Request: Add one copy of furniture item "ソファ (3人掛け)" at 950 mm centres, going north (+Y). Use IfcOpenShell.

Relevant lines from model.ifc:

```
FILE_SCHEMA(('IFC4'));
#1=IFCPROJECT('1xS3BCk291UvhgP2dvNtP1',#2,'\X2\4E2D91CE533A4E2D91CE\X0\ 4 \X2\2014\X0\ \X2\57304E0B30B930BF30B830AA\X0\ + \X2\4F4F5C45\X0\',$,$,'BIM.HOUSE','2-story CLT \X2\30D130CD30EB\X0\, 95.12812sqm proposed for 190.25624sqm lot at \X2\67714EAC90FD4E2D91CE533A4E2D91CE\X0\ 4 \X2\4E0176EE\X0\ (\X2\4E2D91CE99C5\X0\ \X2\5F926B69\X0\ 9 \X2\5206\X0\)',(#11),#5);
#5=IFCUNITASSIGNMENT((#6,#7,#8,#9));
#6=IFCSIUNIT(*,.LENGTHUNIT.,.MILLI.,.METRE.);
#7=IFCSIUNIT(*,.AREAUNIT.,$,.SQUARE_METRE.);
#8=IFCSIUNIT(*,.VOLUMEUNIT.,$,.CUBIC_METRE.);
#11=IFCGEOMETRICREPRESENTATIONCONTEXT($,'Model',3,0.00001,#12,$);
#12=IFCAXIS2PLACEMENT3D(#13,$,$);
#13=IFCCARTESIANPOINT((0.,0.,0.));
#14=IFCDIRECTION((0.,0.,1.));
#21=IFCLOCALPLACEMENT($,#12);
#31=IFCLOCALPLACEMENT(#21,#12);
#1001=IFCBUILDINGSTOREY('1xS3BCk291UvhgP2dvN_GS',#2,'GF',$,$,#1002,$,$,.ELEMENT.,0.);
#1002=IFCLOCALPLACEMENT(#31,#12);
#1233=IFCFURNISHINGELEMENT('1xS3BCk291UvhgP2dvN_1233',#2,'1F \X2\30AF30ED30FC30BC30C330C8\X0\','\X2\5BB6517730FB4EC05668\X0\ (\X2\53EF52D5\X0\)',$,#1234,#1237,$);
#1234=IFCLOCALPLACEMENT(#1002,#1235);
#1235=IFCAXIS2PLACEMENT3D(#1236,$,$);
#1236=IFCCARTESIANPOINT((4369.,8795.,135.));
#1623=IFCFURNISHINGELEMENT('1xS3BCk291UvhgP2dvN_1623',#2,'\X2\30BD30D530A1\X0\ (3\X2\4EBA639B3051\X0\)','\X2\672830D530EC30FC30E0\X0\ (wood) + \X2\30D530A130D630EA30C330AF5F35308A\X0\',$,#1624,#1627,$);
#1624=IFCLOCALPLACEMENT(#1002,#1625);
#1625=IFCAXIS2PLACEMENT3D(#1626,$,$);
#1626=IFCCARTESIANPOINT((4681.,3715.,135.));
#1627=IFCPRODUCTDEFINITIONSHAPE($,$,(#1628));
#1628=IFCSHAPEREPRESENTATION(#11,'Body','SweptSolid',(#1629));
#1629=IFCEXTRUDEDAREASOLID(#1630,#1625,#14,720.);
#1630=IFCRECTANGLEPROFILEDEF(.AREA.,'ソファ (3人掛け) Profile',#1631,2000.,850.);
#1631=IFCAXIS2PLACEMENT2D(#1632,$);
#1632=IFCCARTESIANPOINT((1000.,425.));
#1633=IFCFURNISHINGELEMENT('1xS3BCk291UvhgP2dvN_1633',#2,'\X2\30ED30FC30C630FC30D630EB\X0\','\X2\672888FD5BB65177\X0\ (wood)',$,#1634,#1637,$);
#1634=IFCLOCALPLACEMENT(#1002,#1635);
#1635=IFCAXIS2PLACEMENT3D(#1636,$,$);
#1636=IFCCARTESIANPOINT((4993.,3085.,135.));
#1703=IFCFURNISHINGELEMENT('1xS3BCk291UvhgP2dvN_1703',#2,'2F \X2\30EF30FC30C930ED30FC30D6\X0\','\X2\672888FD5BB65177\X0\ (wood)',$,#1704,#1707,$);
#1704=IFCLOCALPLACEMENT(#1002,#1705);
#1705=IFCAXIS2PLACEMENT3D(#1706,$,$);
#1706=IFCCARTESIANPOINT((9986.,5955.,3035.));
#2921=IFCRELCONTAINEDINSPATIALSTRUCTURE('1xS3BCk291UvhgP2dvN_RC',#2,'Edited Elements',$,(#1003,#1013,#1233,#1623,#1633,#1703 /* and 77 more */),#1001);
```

```python
import numpy as np
import ifcopenshell
import ifcopenshell.api.geometry
import ifcopenshell.api.root
import ifcopenshell.util.element
import ifcopenshell.util.placement

model = ifcopenshell.open("model.ifc")


def reuse_history(source, copy):
    """copy_class also copies each property set's owner history, people and application; keep the originals."""
    for rel in copy.IsDefinedBy:
        if rel.is_a("IfcRelDefinesByProperties") and (history := rel.RelatingPropertyDefinition.OwnerHistory):
            rel.RelatingPropertyDefinition.OwnerHistory = source.OwnerHistory
            ifcopenshell.util.element.remove_deep2(model, history)


source = model.by_guid("1xS3BCk291UvhgP2dvN_1623")
base = ifcopenshell.util.placement.get_local_placement(source.ObjectPlacement)
step = np.array([0.0, 1.0, 0.0]) * 950.0

for i in range(1, 2):
    copy = ifcopenshell.api.root.copy_class(model, product=source)
    copy.Representation = ifcopenshell.util.element.copy_deep(
        model, source.Representation, exclude=["IfcGeometricRepresentationContext", "IfcRepresentationMap"]
    )
    reuse_history(source, copy)
    matrix = base.copy()
    matrix[:3, 3] += i * step
    print("added at", matrix[:3, 3].round(3) + 0.0)
    ifcopenshell.api.geometry.edit_object_placement(model, product=copy, matrix=matrix, is_si=False)

model.write("model-out.ifc")
```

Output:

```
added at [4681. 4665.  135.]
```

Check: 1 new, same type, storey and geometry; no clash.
